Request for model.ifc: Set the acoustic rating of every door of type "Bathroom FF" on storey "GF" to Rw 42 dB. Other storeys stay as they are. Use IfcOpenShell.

First a look at what the model holds.

```python
import ifcopenshell
import ifcopenshell.util.element

model = ifcopenshell.open("model.ifc")
print(model.schema)
storey = next(s for s in model.by_type("IfcBuildingStorey") if s.Name == "GF")
doors = [e for e in ifcopenshell.util.element.get_decomposition(storey) if e.is_a("IfcDoor")]
seen = {}
for e in doors:
    element_type = ifcopenshell.util.element.get_type(e)
    key = (element_type.Name if element_type != e and element_type else None, ifcopenshell.util.element.get_pset(e, "Pset_DoorCommon", "AcousticRating"))
    seen[key] = seen.get(key, 0) + 1
for (name, value), count in sorted(seen.items(), key=str):
    print(count, "x", name, "|", value)
```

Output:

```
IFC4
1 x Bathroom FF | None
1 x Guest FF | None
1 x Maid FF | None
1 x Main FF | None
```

```python
import ifcopenshell
import ifcopenshell.api.pset
import ifcopenshell.util.element

model = ifcopenshell.open("model.ifc")

storey = next(s for s in model.by_type("IfcBuildingStorey") if s.Name == "GF")
doors = [e for e in ifcopenshell.util.element.get_decomposition(storey) if e.is_a("IfcDoor")]

count = 0
for e in doors:
    element_type = ifcopenshell.util.element.get_type(e)
    if element_type in (None, e) or element_type.Name != "Bathroom FF":
        continue
    # add_pset returns the element's existing set when there is one.
    pset = ifcopenshell.api.pset.add_pset(model, product=e, name="Pset_DoorCommon")
    ifcopenshell.api.pset.edit_pset(model, pset=pset, properties={"AcousticRating": "Rw 42 dB"})
    count += 1

print(count, "doors updated")

model.write("model_updated.ifc")
```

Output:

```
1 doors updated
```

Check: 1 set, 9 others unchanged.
